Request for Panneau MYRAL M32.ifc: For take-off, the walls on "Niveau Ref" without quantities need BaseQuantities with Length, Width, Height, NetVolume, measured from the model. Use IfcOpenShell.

First a look at what the model holds.

```python
import ifcopenshell
import ifcopenshell.util.element
import ifcopenshell.util.unit

model = ifcopenshell.open("Panneau MYRAL M32.ifc")
print(model.schema)
for unit_type in ("LENGTHUNIT", "AREAUNIT", "VOLUMEUNIT"):
    print(unit_type, ifcopenshell.util.unit.calculate_unit_scale(model, unit_type))
storey = next(s for s in model.by_type("IfcBuildingStorey") if s.Name == "Niveau Ref")
walls = [e for e in ifcopenshell.util.element.get_decomposition(storey) if e.is_a("IfcWall")]
for e in sorted(walls, key=lambda e: e.id()):
    print(e.id(), e.is_a(), e.Name, list(ifcopenshell.util.element.get_psets(e, qtos_only=True)), sep=" | ")
```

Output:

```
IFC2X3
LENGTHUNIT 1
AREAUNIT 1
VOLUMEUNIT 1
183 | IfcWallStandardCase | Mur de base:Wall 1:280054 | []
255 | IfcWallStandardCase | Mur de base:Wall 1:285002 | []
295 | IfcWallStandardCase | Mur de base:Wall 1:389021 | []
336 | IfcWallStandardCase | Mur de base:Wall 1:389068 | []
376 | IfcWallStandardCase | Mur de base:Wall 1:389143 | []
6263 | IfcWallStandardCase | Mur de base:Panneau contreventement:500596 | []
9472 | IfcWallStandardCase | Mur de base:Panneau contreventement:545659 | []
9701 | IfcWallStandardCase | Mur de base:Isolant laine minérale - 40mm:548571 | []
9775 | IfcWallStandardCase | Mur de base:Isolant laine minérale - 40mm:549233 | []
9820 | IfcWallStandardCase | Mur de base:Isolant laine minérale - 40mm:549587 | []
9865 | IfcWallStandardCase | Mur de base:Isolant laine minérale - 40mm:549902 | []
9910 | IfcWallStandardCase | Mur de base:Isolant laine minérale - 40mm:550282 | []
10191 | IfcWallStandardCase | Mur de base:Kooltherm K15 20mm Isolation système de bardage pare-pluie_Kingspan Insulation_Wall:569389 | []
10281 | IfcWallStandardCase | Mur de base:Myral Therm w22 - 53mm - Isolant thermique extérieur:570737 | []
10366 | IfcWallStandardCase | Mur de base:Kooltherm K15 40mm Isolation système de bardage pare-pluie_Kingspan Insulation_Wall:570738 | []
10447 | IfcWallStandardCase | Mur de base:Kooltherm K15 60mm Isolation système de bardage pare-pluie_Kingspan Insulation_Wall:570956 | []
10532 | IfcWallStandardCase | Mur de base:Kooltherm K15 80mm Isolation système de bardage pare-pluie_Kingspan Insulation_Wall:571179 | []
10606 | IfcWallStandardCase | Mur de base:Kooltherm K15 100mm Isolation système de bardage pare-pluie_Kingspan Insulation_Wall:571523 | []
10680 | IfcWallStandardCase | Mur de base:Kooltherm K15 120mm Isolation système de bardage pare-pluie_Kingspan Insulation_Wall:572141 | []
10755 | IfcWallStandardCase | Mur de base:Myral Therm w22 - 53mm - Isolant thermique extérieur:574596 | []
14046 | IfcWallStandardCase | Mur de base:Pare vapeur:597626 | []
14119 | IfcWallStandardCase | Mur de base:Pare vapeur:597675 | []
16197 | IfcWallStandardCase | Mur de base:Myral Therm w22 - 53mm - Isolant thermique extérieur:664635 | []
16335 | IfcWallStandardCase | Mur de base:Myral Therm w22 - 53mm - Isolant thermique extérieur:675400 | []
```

```python
import ifcopenshell
import ifcopenshell.api.pset
import ifcopenshell.geom
import ifcopenshell.util.element
import ifcopenshell.util.shape
import ifcopenshell.util.unit

model = ifcopenshell.open("Panneau MYRAL M32.ifc")
unit_scale = ifcopenshell.util.unit.calculate_unit_scale(model)
volume_scale = ifcopenshell.util.unit.calculate_unit_scale(model, "VOLUMEUNIT")
settings = ifcopenshell.geom.settings()

storey = next(s for s in model.by_type("IfcBuildingStorey") if s.Name == "Niveau Ref")
walls = [e for e in ifcopenshell.util.element.get_decomposition(storey) if e.is_a("IfcWall")]

for e in sorted(walls, key=lambda e: e.id()):
    if ifcopenshell.util.element.get_psets(e, qtos_only=True, should_inherit=False):
        continue
    # Geometry comes back in metres, in the element's own axes.
    shape = ifcopenshell.geom.create_shape(settings, e)
    values = {
        "Length": ifcopenshell.util.shape.get_x(shape.geometry) / unit_scale,
        "Width": ifcopenshell.util.shape.get_y(shape.geometry) / unit_scale,
        "Height": ifcopenshell.util.shape.get_z(shape.geometry) / unit_scale,
        "NetVolume": ifcopenshell.util.shape.get_volume(shape.geometry) / volume_scale,
    }
    qto = ifcopenshell.api.pset.add_qto(model, product=e, name="BaseQuantities")
    ifcopenshell.api.pset.edit_qto(model, qto=qto, properties=values)
    print(e.id(), {k: round(v, 3) for k, v in values.items()})

model.write("Panneau MYRAL M32_edited.ifc")
```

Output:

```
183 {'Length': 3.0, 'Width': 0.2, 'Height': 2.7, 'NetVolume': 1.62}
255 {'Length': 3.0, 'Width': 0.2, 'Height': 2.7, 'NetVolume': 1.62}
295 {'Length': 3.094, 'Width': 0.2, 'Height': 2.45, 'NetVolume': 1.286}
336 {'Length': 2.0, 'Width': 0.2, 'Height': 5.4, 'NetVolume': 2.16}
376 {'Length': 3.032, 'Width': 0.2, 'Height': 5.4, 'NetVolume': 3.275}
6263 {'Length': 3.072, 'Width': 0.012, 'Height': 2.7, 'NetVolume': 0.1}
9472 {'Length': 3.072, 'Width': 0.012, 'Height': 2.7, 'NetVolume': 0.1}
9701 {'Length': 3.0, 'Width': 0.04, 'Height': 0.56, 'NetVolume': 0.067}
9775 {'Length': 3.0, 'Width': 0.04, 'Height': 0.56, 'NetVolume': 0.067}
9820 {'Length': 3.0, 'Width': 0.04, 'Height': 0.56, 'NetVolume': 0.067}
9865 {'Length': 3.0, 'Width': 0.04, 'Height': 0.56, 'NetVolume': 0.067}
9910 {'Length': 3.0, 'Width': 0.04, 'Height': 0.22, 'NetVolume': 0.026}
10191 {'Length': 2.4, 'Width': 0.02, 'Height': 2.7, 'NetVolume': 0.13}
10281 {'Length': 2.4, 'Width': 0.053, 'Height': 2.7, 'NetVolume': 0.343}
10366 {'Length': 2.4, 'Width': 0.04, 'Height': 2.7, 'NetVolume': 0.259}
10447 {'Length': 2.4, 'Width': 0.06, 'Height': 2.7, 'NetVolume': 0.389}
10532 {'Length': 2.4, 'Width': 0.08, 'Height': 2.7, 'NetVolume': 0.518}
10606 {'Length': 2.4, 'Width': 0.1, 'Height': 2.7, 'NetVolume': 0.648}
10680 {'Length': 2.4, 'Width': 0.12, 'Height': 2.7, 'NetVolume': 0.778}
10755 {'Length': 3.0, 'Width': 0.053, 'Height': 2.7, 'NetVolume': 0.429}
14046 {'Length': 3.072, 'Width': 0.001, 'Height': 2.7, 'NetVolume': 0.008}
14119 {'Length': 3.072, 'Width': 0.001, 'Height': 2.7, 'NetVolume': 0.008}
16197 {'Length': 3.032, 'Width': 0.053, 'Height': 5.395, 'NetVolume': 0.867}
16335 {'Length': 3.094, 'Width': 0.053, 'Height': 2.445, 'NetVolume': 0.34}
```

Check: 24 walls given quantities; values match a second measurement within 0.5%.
